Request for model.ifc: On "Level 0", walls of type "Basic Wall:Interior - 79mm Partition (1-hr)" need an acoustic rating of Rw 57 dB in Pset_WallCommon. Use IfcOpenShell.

First a look at what the model holds.

```python
import ifcopenshell
import ifcopenshell.util.element

model = ifcopenshell.open("model.ifc")
print(model.schema)
storey = next(s for s in model.by_type("IfcBuildingStorey") if s.Name == "Level 0")
walls = [e for e in ifcopenshell.util.element.get_decomposition(storey) if e.is_a("IfcWall")]
seen = {}
for e in walls:
    element_type = ifcopenshell.util.element.get_type(e)
    key = (element_type.Name if element_type != e and element_type else None, ifcopenshell.util.element.get_pset(e, "Pset_WallCommon", "AcousticRating"))
    seen[key] = seen.get(key, 0) + 1
for (name, value), count in sorted(seen.items(), key=str):
    print(count, "x", name, "|", value)
```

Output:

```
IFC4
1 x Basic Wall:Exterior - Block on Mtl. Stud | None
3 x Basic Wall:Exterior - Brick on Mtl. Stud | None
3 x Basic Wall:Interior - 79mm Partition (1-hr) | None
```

```python
import ifcopenshell
import ifcopenshell.api.pset
import ifcopenshell.util.element

model = ifcopenshell.open("model.ifc")

storey = next(s for s in model.by_type("IfcBuildingStorey") if s.Name == "Level 0")
walls = [e for e in ifcopenshell.util.element.get_decomposition(storey) if e.is_a("IfcWall")]

count = 0
for e in walls:
    element_type = ifcopenshell.util.element.get_type(e)
    if element_type in (None, e) or element_type.Name != "Basic Wall:Interior - 79mm Partition (1-hr)":
        continue
    # add_pset returns the element's existing set when there is one.
    pset = ifcopenshell.api.pset.add_pset(model, product=e, name="Pset_WallCommon")
    ifcopenshell.api.pset.edit_pset(model, pset=pset, properties={"AcousticRating": "Rw 57 dB"})
    count += 1

print(count, "walls updated")

model.write("model_v2.ifc")
```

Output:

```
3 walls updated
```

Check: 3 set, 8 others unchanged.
